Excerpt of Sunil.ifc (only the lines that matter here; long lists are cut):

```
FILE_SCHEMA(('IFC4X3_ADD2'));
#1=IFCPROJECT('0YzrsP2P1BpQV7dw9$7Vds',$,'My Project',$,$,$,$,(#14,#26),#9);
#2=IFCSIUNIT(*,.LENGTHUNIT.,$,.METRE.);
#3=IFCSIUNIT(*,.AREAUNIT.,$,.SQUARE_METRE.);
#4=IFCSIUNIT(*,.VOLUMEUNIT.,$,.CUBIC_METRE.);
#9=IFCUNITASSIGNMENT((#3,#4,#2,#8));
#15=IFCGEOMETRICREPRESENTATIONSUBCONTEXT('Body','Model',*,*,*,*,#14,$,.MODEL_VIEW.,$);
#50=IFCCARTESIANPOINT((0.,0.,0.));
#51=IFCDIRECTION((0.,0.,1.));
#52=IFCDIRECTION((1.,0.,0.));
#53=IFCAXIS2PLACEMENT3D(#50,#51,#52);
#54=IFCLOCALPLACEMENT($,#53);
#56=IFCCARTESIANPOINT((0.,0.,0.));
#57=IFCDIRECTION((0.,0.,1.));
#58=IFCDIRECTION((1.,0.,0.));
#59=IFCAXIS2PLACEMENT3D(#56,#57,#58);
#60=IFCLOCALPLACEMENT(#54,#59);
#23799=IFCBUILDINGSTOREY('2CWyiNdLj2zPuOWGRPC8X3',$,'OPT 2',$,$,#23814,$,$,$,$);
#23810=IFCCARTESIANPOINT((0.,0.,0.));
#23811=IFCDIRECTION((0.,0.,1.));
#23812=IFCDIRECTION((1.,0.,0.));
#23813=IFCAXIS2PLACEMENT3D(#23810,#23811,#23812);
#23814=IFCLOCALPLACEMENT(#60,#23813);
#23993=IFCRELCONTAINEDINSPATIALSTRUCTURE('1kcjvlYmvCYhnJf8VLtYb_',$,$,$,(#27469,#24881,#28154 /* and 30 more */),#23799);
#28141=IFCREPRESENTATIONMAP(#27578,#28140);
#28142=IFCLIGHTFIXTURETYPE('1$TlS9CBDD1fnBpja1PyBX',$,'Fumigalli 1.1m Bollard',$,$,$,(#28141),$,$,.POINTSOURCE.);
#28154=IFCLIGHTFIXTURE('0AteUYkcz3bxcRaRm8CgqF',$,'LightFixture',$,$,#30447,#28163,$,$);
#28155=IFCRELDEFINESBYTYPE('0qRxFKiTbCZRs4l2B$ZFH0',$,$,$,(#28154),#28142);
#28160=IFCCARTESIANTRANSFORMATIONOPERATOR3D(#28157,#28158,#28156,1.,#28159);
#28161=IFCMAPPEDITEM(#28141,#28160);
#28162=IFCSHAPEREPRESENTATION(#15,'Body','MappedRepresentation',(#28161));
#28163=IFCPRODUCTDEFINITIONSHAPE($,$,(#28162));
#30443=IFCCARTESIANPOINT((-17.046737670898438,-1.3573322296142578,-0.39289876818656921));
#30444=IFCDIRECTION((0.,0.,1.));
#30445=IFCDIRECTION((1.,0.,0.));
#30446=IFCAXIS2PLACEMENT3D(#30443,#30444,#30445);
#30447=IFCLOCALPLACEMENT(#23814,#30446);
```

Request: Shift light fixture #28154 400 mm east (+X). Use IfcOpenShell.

```python
import ifcopenshell
import ifcopenshell.api.geometry
import ifcopenshell.util.placement
import ifcopenshell.util.unit

model = ifcopenshell.open("Sunil.ifc")
unit_scale = ifcopenshell.util.unit.calculate_unit_scale(model)

item = model.by_guid("0AteUYkcz3bxcRaRm8CgqF")
matrix = ifcopenshell.util.placement.get_local_placement(item.ObjectPlacement)
matrix[0, 3] += 0.4 / unit_scale
ifcopenshell.api.geometry.edit_object_placement(model, product=item, matrix=matrix, is_si=False)

print(ifcopenshell.util.placement.get_local_placement(item.ObjectPlacement).round(3) + 0.0)

model.write("Sunil_v2.ifc")
```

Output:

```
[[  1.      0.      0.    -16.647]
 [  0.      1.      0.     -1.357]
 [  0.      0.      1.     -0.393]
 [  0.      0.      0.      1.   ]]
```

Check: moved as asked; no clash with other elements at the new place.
